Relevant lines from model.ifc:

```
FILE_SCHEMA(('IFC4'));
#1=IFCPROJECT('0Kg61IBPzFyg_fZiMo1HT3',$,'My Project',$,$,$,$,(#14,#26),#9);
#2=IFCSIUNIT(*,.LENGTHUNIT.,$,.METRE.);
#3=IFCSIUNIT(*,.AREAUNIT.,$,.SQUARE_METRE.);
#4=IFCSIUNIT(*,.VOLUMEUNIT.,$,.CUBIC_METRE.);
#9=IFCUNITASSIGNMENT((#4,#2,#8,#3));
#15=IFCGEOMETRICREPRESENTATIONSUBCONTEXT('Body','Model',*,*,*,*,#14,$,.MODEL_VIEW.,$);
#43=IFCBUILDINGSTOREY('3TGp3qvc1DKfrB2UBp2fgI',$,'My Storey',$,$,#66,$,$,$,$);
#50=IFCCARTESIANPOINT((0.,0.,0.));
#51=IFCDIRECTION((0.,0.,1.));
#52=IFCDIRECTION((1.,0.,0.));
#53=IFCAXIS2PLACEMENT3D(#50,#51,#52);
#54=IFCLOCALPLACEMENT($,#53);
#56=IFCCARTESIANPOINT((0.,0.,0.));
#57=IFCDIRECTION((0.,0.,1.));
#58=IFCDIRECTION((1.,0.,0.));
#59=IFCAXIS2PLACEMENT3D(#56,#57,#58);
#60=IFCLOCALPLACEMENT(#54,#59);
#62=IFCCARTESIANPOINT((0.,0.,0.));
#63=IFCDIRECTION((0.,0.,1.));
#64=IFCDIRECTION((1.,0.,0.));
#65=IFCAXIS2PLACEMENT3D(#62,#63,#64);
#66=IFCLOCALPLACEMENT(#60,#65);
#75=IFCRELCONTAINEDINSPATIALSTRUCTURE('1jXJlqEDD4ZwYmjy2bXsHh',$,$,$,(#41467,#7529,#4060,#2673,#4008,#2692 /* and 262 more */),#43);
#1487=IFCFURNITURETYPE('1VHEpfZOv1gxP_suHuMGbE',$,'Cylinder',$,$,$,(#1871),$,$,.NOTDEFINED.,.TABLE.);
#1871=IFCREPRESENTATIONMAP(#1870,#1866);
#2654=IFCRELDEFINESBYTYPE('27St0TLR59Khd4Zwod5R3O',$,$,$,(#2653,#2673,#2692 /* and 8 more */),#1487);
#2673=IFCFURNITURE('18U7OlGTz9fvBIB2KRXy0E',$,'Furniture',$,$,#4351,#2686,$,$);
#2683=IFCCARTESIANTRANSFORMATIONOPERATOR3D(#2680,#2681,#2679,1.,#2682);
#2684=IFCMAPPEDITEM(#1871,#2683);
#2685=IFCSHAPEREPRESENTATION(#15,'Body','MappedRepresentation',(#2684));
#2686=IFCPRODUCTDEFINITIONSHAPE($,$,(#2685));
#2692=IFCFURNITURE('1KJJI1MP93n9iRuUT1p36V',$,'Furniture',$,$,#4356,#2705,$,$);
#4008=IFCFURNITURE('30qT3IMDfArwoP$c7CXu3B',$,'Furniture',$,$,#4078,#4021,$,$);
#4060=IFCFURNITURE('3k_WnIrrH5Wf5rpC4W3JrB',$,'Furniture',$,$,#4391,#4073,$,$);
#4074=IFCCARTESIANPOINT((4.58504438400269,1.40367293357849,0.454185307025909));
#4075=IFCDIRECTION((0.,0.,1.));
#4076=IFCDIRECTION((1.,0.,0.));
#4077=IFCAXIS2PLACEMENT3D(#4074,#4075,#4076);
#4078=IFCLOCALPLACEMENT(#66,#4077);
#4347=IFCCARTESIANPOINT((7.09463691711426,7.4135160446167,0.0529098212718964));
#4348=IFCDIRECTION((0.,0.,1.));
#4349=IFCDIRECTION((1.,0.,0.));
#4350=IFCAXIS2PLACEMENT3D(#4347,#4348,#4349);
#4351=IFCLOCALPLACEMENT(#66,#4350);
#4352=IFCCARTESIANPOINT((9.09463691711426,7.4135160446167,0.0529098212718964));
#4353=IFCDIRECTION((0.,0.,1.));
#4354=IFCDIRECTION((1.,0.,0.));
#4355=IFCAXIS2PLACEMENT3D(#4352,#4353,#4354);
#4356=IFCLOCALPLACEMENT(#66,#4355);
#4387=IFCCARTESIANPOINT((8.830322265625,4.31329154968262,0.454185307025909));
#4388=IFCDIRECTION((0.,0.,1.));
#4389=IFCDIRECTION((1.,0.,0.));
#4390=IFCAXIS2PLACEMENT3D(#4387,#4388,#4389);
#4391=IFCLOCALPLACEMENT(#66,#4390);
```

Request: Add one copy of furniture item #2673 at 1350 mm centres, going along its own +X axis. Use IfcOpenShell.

```python
import ifcopenshell
import ifcopenshell.api.geometry
import ifcopenshell.api.root
import ifcopenshell.util.element
import ifcopenshell.util.placement
import ifcopenshell.util.unit

model = ifcopenshell.open("model.ifc")
unit_scale = ifcopenshell.util.unit.calculate_unit_scale(model)

source = model.by_guid("18U7OlGTz9fvBIB2KRXy0E")
base = ifcopenshell.util.placement.get_local_placement(source.ObjectPlacement)
step = base[:3, 0] * 1.35 / unit_scale

for i in range(1, 2):
    copy = ifcopenshell.api.root.copy_class(model, product=source)
    copy.Representation = ifcopenshell.util.element.copy_deep(
        model, source.Representation, exclude=["IfcGeometricRepresentationContext", "IfcRepresentationMap"]
    )
    matrix = base.copy()
    matrix[:3, 3] += i * step
    print("added at", matrix[:3, 3].round(3) + 0.0)
    ifcopenshell.api.geometry.edit_object_placement(model, product=copy, matrix=matrix, is_si=False)

model.write("model_v2.ifc")
```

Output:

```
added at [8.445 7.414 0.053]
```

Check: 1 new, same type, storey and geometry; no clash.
